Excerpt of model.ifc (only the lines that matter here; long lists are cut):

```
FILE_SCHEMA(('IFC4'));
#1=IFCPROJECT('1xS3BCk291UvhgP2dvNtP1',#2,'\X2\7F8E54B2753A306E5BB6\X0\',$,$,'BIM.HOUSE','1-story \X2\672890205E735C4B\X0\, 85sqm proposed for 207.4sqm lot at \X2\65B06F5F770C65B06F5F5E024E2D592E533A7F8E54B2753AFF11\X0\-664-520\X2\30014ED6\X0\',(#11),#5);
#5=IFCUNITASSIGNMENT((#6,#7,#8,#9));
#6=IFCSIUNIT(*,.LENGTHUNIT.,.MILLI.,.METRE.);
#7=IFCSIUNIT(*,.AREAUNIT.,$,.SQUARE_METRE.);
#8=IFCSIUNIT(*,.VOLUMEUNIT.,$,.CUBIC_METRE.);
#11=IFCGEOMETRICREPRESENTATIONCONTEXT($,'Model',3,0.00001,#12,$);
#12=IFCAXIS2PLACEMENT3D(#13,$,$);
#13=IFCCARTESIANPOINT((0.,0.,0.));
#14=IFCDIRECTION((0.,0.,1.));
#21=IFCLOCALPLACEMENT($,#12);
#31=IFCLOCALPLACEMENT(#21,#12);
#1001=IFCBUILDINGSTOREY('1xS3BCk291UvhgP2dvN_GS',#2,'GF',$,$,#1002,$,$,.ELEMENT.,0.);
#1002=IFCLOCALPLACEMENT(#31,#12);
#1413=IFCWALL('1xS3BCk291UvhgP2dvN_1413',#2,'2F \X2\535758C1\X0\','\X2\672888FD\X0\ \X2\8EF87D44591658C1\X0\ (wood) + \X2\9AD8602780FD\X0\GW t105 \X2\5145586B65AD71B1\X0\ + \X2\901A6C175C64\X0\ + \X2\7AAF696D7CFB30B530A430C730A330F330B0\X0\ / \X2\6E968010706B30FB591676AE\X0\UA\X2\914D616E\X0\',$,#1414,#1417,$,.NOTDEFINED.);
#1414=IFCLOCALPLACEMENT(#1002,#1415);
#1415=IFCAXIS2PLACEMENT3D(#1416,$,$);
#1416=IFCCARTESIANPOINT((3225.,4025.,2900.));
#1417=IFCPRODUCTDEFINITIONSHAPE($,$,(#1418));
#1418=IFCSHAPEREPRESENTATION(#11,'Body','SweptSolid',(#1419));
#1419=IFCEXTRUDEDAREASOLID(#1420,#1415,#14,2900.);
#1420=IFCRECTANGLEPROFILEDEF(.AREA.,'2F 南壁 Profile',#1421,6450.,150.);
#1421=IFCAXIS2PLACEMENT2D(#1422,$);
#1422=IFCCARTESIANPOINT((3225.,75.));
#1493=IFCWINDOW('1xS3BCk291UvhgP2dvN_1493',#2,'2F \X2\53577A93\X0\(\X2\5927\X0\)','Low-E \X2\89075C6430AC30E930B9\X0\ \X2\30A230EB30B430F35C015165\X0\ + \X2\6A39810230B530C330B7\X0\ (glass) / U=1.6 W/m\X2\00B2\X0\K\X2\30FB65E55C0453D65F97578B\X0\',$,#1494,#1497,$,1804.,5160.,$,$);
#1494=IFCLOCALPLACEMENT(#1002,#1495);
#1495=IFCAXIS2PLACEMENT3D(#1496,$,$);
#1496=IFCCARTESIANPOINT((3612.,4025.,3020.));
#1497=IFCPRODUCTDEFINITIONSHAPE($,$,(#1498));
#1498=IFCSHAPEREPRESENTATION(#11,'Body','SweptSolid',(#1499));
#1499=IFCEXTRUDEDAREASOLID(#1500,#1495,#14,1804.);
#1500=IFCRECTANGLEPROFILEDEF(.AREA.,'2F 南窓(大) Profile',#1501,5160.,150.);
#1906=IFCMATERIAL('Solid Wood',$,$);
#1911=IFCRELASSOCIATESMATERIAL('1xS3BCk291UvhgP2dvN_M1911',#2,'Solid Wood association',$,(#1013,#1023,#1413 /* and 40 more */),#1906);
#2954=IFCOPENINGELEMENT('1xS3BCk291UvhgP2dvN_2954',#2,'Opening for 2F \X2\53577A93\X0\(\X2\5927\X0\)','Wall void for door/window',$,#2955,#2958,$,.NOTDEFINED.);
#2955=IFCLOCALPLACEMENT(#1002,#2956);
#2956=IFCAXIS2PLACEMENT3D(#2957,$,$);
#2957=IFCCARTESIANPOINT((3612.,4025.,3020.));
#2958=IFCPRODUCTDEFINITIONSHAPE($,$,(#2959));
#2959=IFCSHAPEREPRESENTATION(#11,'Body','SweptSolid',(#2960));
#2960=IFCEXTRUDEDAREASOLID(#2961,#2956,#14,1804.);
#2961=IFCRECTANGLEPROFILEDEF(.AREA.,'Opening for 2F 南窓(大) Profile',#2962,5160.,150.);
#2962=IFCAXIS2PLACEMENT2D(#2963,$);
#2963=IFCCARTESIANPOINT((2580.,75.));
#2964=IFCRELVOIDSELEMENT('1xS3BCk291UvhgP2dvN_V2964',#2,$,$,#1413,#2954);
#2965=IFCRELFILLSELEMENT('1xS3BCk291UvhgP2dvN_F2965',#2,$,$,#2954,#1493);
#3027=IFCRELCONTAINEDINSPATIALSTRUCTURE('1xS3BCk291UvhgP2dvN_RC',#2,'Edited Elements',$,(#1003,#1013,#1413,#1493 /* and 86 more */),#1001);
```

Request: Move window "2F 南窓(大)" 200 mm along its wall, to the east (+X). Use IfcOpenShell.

```python
import ifcopenshell
import ifcopenshell.api.geometry
import ifcopenshell.util.placement

model = ifcopenshell.open("model.ifc")

window = model.by_guid("1xS3BCk291UvhgP2dvN_1493")
opening = window.FillsVoids[0].RelatingOpeningElement
wall = opening.VoidsElements[0].RelatingBuildingElement

wall_matrix = ifcopenshell.util.placement.get_local_placement(wall.ObjectPlacement)
shift = wall_matrix[:3, 0] * 200.0
before = ifcopenshell.util.placement.get_local_placement(window.ObjectPlacement)[:3, 3].copy()

# The window is not placed relative to its opening, so move both.
for product in (opening, window):
    matrix = ifcopenshell.util.placement.get_local_placement(product.ObjectPlacement)
    matrix[:3, 3] += shift
    ifcopenshell.api.geometry.edit_object_placement(model, product=product, matrix=matrix, is_si=False)

after = ifcopenshell.util.placement.get_local_placement(window.ObjectPlacement)[:3, 3]
print("window moved by", (after - before).round(3) + 0.0)

model.write("model_updated.ifc")
```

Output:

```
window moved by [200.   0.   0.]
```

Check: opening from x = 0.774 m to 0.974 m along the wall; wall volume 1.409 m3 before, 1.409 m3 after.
